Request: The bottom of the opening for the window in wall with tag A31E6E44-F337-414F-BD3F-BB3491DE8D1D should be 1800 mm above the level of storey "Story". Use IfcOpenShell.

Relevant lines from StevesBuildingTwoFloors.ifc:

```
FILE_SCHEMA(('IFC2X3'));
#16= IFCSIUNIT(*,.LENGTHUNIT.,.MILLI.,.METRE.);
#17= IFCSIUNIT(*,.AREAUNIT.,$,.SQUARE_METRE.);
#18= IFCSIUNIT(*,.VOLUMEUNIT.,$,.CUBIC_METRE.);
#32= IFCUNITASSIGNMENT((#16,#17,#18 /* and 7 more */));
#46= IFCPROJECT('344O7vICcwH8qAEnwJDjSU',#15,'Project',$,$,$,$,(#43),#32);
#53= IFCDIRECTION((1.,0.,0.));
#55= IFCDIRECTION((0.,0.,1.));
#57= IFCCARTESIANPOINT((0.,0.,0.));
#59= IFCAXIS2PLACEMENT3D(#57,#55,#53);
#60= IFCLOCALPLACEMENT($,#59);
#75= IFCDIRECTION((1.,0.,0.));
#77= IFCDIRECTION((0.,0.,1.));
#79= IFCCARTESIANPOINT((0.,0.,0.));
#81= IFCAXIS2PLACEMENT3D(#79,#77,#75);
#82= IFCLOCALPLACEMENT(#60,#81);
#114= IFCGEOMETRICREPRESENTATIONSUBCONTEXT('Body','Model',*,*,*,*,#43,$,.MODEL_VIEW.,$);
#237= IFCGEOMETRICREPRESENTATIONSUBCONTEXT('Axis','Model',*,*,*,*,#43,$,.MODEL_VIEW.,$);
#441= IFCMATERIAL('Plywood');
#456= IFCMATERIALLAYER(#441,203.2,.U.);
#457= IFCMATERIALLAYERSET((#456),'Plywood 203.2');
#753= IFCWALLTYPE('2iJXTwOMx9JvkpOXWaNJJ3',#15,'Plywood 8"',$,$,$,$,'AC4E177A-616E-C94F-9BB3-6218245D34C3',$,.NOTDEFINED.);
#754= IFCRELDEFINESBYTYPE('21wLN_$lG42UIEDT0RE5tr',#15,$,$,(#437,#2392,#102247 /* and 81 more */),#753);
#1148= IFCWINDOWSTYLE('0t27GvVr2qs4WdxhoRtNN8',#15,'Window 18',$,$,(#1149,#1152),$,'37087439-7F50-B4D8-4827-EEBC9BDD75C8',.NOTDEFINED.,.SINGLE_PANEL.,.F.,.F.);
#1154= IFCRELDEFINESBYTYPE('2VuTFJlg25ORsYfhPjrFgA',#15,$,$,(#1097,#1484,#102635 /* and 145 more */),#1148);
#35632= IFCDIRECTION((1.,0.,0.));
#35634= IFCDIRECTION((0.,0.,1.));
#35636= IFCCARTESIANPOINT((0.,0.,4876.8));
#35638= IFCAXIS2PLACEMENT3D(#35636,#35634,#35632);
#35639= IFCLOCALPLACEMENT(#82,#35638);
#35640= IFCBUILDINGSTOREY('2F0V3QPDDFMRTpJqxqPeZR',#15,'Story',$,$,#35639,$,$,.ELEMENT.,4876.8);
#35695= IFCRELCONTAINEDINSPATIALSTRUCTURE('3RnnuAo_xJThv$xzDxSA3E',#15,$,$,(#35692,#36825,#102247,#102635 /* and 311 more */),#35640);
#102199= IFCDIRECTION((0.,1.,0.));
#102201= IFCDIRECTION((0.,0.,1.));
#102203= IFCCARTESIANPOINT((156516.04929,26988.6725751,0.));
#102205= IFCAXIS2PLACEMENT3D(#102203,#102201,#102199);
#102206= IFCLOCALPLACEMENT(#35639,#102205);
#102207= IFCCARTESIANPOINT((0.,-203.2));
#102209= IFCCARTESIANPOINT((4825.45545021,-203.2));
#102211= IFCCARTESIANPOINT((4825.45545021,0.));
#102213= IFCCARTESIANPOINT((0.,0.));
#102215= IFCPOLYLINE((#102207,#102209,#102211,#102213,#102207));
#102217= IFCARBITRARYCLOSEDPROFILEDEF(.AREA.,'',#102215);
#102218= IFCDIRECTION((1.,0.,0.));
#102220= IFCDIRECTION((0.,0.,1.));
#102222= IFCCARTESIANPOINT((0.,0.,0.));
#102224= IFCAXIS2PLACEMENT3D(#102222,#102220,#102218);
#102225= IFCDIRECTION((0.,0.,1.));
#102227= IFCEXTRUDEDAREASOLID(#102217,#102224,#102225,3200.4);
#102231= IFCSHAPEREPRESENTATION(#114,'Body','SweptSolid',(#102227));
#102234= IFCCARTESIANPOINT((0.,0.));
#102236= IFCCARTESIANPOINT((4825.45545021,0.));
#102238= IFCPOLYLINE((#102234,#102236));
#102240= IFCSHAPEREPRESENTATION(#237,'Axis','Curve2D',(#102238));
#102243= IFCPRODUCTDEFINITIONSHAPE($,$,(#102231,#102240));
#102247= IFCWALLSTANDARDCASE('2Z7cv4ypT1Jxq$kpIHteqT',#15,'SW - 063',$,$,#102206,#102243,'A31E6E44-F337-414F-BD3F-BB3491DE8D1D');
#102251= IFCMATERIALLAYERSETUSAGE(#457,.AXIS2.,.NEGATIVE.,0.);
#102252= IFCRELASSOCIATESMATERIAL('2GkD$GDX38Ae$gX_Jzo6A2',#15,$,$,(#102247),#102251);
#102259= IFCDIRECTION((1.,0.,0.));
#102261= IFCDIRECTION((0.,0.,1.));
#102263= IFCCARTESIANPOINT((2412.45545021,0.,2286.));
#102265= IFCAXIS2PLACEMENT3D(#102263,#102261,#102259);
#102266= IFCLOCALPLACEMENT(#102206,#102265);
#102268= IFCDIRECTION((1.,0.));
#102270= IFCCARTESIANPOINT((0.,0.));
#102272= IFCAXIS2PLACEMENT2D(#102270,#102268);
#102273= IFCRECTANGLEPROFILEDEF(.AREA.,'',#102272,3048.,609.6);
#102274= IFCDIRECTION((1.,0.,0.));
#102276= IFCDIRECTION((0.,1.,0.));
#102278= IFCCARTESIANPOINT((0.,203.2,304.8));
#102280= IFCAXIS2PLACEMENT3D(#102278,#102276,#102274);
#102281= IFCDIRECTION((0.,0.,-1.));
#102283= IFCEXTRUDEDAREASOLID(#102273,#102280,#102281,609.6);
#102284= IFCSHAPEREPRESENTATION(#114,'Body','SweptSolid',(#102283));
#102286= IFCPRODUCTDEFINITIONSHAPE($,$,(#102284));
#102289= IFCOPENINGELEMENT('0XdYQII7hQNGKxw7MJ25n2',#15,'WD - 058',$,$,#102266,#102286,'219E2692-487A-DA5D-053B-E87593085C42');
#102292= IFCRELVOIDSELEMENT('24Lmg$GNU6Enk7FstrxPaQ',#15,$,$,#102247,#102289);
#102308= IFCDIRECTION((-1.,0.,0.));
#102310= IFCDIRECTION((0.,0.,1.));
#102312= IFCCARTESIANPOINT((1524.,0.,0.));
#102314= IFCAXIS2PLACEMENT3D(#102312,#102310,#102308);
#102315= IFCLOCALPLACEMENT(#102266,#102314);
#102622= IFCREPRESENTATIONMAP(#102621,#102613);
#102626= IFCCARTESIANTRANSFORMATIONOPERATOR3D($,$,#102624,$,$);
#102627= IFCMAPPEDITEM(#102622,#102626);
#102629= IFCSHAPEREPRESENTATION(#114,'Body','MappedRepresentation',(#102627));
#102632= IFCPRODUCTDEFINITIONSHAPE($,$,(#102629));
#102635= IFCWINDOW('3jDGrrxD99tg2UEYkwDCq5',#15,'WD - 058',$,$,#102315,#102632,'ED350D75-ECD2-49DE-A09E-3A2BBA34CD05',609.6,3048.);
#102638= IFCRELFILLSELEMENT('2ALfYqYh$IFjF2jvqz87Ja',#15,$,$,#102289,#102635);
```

```python
import numpy as np
import ifcopenshell
import ifcopenshell.api.geometry
import ifcopenshell.geom
import ifcopenshell.util.element
import ifcopenshell.util.placement
import ifcopenshell.util.shape
import ifcopenshell.util.unit

model = ifcopenshell.open("StevesBuildingTwoFloors.ifc")
unit_scale = ifcopenshell.util.unit.calculate_unit_scale(model)

window = model.by_id(102635)
opening = window.FillsVoids[0].RelatingOpeningElement
storey = ifcopenshell.util.element.get_container(window, ifc_class="IfcBuildingStorey")
level = ifcopenshell.util.placement.get_local_placement(storey.ObjectPlacement)[2, 3]

# The opening's origin need not be at the sill, so measure its lowest point.
shape = ifcopenshell.geom.create_shape(ifcopenshell.geom.settings(), opening)
bottom = ifcopenshell.util.shape.get_shape_bottom_elevation(shape, shape.geometry) / unit_scale
dz = level + 1.8 / unit_scale - bottom

shift = np.array([0.0, 0.0, dz])
# The window is placed relative to its opening, so it follows when the opening moves.
matrix = ifcopenshell.util.placement.get_local_placement(opening.ObjectPlacement)
matrix[:3, 3] += shift
ifcopenshell.api.geometry.edit_object_placement(
    model, product=opening, matrix=matrix, is_si=False, should_transform_children=True
)

print(f"moved by {dz * unit_scale:+.3f} m")

model.write("StevesBuildingTwoFloors_v2.ifc")
```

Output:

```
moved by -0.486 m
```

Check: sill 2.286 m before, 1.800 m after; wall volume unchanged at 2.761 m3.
